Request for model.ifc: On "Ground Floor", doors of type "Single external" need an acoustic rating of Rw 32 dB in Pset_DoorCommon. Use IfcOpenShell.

First a look at what the model holds.

```python
import ifcopenshell
import ifcopenshell.util.element

model = ifcopenshell.open("model.ifc")
print(model.schema)
storey = next(s for s in model.by_type("IfcBuildingStorey") if s.Name == "Ground Floor")
doors = [e for e in ifcopenshell.util.element.get_decomposition(storey) if e.is_a("IfcDoor")]
seen = {}
for e in doors:
    element_type = ifcopenshell.util.element.get_type(e)
    key = (element_type.Name if element_type != e and element_type else None, ifcopenshell.util.element.get_pset(e, "Pset_DoorCommon", "AcousticRating"))
    seen[key] = seen.get(key, 0) + 1
for (name, value), count in sorted(seen.items(), key=str):
    print(count, "x", name, "|", value)
```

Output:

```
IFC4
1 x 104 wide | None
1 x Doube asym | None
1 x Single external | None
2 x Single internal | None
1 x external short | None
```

```python
import ifcopenshell
import ifcopenshell.api.pset
import ifcopenshell.util.element

model = ifcopenshell.open("model.ifc")

storey = next(s for s in model.by_type("IfcBuildingStorey") if s.Name == "Ground Floor")
doors = [e for e in ifcopenshell.util.element.get_decomposition(storey) if e.is_a("IfcDoor")]

count = 0
for e in doors:
    element_type = ifcopenshell.util.element.get_type(e)
    if element_type in (None, e) or element_type.Name != "Single external":
        continue
    # add_pset returns the element's existing set when there is one.
    pset = ifcopenshell.api.pset.add_pset(model, product=e, name="Pset_DoorCommon")
    ifcopenshell.api.pset.edit_pset(model, pset=pset, properties={"AcousticRating": "Rw 32 dB"})
    count += 1

print(count, "doors updated")

model.write("model_edited.ifc")
```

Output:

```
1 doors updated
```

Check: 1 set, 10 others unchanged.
